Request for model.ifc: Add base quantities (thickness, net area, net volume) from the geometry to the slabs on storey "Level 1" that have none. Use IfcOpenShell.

First a look at what the model holds.

```python
import ifcopenshell
import ifcopenshell.util.element
import ifcopenshell.util.unit

model = ifcopenshell.open("model.ifc")
print(model.schema)
for unit_type in ("LENGTHUNIT", "AREAUNIT", "VOLUMEUNIT"):
    print(unit_type, ifcopenshell.util.unit.calculate_unit_scale(model, unit_type))
storey = next(s for s in model.by_type("IfcBuildingStorey") if s.Name == "Level 1")
slabs = [e for e in ifcopenshell.util.element.get_decomposition(storey) if e.is_a("IfcSlab")]
for e in sorted(slabs, key=lambda e: e.id()):
    print(e.id(), e.is_a(), e.Name, list(ifcopenshell.util.element.get_psets(e, qtos_only=True)), sep=" | ")
```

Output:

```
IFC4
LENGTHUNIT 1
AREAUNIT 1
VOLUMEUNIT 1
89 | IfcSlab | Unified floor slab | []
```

```python
import ifcopenshell
import ifcopenshell.api.pset
import ifcopenshell.geom
import ifcopenshell.util.element
import ifcopenshell.util.shape
import ifcopenshell.util.unit

model = ifcopenshell.open("model.ifc")
unit_scale = ifcopenshell.util.unit.calculate_unit_scale(model)
area_scale = ifcopenshell.util.unit.calculate_unit_scale(model, "AREAUNIT")
volume_scale = ifcopenshell.util.unit.calculate_unit_scale(model, "VOLUMEUNIT")
settings = ifcopenshell.geom.settings()

storey = next(s for s in model.by_type("IfcBuildingStorey") if s.Name == "Level 1")
slabs = [e for e in ifcopenshell.util.element.get_decomposition(storey) if e.is_a("IfcSlab")]

for e in sorted(slabs, key=lambda e: e.id()):
    if ifcopenshell.util.element.get_psets(e, qtos_only=True, should_inherit=False):
        continue
    # Geometry comes back in metres, in the element's own axes.
    shape = ifcopenshell.geom.create_shape(settings, e)
    values = {
        "Width": ifcopenshell.util.shape.get_z(shape.geometry) / unit_scale,
        "NetArea": ifcopenshell.util.shape.get_footprint_area(shape.geometry) / area_scale,
        "NetVolume": ifcopenshell.util.shape.get_volume(shape.geometry) / volume_scale,
    }
    qto = ifcopenshell.api.pset.add_qto(model, product=e, name="Qto_SlabBaseQuantities")
    ifcopenshell.api.pset.edit_qto(model, qto=qto, properties=values)
    print(e.id(), {k: round(v, 3) for k, v in values.items()})

model.write("model_v2.ifc")
```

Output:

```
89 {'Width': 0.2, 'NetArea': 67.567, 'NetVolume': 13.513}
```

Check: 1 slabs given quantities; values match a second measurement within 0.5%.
